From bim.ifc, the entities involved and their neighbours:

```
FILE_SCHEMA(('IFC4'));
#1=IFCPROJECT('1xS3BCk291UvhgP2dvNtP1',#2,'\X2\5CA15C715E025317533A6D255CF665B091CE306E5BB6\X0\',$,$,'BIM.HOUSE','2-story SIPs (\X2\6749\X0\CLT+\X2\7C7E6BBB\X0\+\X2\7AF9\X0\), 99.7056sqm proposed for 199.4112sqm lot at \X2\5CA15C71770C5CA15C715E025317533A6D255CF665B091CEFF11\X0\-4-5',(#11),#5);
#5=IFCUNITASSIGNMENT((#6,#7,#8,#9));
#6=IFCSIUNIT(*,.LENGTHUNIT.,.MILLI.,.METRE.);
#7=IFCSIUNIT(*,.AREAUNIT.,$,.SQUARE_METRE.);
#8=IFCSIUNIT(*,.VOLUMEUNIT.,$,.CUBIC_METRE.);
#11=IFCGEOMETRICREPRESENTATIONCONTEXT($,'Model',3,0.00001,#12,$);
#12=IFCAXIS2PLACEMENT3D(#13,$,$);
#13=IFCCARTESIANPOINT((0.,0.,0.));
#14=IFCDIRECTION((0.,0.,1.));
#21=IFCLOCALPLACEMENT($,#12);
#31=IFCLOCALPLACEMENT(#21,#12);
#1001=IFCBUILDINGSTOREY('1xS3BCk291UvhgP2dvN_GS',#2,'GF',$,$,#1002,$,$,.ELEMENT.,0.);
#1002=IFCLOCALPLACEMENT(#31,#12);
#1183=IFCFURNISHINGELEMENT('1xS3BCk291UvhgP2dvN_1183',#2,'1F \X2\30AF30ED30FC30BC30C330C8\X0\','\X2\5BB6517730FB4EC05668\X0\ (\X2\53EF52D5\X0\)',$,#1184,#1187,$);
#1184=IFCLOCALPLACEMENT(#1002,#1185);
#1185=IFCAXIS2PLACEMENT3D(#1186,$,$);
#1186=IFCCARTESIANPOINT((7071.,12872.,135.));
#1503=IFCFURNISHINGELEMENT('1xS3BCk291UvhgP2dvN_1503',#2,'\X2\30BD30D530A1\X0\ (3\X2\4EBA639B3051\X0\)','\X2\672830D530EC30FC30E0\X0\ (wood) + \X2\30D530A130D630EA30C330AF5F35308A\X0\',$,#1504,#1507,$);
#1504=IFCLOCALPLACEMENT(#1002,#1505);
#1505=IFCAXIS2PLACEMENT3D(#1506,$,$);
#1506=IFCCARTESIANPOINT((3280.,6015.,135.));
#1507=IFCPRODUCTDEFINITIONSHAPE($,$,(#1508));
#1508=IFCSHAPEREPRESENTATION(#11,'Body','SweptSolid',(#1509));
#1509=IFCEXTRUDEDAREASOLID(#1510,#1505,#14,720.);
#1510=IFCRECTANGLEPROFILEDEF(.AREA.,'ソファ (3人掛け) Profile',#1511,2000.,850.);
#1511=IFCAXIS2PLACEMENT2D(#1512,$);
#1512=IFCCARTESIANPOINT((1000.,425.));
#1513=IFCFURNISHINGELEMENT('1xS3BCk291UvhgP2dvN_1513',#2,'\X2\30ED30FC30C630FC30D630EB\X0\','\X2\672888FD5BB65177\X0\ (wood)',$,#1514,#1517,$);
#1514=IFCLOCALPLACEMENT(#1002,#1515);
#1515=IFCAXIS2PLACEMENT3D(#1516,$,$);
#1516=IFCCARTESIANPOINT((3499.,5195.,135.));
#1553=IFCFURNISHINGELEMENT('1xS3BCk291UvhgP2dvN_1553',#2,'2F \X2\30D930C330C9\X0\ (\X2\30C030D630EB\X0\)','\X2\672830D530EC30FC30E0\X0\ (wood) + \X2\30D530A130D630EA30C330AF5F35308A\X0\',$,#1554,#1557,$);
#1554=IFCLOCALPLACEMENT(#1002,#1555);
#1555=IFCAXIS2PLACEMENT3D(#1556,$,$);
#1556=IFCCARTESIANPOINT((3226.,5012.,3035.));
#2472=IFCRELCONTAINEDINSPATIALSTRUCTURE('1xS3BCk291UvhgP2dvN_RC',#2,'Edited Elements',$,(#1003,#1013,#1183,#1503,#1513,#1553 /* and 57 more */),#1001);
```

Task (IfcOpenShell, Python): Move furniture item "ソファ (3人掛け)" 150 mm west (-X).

```python
import ifcopenshell
import ifcopenshell.api.geometry
import ifcopenshell.util.placement

model = ifcopenshell.open("bim.ifc")

item = model.by_id(1503)
matrix = ifcopenshell.util.placement.get_local_placement(item.ObjectPlacement)
matrix[0, 3] -= 150.0
ifcopenshell.api.geometry.edit_object_placement(model, product=item, matrix=matrix, is_si=False)

print(ifcopenshell.util.placement.get_local_placement(item.ObjectPlacement).round(3) + 0.0)

model.write("bim_rev.ifc")
```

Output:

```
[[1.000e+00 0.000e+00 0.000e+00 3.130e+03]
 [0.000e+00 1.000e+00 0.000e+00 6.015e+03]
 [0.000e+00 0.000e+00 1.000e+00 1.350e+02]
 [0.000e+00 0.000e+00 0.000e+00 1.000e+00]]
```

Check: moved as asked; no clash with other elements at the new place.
